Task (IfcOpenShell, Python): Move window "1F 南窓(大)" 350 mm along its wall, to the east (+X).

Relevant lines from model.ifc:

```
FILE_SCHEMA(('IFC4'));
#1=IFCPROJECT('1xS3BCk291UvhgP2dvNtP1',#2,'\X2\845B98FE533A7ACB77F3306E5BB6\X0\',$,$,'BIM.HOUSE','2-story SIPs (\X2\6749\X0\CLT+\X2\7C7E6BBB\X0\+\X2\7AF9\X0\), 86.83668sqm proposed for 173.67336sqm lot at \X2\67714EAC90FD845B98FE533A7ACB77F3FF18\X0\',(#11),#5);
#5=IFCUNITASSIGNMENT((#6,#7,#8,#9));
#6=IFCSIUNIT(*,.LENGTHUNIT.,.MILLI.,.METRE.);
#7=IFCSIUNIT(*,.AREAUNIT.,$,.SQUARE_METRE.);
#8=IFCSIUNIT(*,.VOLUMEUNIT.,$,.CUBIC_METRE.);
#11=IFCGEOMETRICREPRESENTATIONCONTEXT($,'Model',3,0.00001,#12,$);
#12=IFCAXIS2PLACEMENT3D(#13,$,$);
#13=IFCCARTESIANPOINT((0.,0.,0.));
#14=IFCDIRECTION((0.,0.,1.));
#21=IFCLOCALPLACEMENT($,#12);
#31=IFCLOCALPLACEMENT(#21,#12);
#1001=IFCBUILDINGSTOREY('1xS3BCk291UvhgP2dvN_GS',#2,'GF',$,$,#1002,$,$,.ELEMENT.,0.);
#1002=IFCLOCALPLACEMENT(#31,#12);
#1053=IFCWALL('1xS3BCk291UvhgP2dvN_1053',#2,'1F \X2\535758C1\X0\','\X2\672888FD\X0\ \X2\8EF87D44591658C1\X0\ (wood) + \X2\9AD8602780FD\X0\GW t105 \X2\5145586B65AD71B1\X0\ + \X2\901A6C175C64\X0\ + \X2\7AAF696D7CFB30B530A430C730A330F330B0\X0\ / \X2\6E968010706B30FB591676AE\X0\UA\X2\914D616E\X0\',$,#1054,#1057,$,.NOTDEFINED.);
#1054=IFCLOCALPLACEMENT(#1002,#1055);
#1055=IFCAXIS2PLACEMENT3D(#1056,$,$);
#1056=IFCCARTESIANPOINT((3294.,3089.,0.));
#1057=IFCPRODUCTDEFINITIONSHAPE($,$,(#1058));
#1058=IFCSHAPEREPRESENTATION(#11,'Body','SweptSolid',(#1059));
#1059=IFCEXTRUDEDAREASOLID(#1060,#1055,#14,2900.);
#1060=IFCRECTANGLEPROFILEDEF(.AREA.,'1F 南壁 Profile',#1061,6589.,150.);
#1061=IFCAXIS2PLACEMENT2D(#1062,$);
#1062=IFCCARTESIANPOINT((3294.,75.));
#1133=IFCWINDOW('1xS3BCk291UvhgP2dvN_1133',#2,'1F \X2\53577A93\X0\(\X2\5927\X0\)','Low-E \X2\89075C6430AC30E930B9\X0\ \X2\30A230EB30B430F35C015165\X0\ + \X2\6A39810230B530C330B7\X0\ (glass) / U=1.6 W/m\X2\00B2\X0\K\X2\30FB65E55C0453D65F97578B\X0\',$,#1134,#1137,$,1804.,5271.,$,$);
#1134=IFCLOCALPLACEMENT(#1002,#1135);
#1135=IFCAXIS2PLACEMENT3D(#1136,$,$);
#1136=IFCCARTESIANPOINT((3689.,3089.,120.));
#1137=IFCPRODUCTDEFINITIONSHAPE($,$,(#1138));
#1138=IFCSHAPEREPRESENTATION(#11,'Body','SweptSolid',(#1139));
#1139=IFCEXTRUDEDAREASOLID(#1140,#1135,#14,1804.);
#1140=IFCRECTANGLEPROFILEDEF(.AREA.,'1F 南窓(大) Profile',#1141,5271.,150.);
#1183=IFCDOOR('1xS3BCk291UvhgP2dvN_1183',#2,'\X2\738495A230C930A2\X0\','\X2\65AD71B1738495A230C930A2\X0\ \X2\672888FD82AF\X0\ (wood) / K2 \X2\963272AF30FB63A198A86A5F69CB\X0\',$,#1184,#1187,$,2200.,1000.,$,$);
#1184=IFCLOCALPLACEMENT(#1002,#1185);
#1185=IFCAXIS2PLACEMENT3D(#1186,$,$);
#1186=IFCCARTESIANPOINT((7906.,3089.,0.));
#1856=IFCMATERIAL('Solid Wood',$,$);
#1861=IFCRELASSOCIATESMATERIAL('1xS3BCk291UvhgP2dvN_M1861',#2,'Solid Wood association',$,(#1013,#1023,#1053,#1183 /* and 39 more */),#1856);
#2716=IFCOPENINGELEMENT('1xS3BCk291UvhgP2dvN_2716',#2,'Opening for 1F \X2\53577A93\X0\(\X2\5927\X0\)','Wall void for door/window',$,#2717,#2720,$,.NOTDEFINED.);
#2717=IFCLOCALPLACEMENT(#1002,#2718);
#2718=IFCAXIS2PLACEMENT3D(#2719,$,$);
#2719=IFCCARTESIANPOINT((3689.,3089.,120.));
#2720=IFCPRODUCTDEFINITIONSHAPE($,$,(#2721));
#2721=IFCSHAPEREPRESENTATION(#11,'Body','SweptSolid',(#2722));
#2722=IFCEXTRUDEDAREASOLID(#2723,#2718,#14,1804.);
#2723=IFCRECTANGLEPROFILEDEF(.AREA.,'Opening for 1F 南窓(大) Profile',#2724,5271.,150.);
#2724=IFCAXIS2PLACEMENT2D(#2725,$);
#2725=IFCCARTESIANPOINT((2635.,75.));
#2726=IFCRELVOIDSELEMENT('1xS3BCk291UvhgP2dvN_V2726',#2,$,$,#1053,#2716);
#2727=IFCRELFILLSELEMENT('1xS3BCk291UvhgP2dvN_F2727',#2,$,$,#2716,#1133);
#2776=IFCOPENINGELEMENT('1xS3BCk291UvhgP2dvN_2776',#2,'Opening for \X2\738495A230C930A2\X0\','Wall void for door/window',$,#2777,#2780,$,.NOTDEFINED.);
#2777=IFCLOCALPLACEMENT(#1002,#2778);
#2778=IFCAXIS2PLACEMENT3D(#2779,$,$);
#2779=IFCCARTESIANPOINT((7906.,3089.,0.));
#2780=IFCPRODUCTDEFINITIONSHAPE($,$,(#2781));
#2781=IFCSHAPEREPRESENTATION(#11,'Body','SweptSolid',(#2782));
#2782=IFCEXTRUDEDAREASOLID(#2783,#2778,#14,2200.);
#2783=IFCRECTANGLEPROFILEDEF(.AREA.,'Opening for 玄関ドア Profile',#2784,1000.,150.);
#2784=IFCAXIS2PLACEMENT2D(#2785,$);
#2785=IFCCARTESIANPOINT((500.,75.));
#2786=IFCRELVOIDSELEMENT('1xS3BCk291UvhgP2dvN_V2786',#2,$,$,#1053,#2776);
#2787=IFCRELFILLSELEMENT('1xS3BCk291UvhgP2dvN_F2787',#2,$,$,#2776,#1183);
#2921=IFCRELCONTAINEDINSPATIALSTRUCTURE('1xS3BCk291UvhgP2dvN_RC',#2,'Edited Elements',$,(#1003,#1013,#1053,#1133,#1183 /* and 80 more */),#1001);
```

```python
import ifcopenshell
import ifcopenshell.api.geometry
import ifcopenshell.util.placement

model = ifcopenshell.open("model.ifc")

window = model.by_guid("1xS3BCk291UvhgP2dvN_1133")
opening = window.FillsVoids[0].RelatingOpeningElement
wall = opening.VoidsElements[0].RelatingBuildingElement

wall_matrix = ifcopenshell.util.placement.get_local_placement(wall.ObjectPlacement)
shift = wall_matrix[:3, 0] * 350.0
before = ifcopenshell.util.placement.get_local_placement(window.ObjectPlacement)[:3, 3].copy()

# The window is not placed relative to its opening, so move both.
for product in (opening, window):
    matrix = ifcopenshell.util.placement.get_local_placement(product.ObjectPlacement)
    matrix[:3, 3] += shift
    ifcopenshell.api.geometry.edit_object_placement(model, product=product, matrix=matrix, is_si=False)

after = ifcopenshell.util.placement.get_local_placement(window.ObjectPlacement)[:3, 3]
print("window moved by", (after - before).round(3) + 0.0)

model.write("model_v2.ifc")
```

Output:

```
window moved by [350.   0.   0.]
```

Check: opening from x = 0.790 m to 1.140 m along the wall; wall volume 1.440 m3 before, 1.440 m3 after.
